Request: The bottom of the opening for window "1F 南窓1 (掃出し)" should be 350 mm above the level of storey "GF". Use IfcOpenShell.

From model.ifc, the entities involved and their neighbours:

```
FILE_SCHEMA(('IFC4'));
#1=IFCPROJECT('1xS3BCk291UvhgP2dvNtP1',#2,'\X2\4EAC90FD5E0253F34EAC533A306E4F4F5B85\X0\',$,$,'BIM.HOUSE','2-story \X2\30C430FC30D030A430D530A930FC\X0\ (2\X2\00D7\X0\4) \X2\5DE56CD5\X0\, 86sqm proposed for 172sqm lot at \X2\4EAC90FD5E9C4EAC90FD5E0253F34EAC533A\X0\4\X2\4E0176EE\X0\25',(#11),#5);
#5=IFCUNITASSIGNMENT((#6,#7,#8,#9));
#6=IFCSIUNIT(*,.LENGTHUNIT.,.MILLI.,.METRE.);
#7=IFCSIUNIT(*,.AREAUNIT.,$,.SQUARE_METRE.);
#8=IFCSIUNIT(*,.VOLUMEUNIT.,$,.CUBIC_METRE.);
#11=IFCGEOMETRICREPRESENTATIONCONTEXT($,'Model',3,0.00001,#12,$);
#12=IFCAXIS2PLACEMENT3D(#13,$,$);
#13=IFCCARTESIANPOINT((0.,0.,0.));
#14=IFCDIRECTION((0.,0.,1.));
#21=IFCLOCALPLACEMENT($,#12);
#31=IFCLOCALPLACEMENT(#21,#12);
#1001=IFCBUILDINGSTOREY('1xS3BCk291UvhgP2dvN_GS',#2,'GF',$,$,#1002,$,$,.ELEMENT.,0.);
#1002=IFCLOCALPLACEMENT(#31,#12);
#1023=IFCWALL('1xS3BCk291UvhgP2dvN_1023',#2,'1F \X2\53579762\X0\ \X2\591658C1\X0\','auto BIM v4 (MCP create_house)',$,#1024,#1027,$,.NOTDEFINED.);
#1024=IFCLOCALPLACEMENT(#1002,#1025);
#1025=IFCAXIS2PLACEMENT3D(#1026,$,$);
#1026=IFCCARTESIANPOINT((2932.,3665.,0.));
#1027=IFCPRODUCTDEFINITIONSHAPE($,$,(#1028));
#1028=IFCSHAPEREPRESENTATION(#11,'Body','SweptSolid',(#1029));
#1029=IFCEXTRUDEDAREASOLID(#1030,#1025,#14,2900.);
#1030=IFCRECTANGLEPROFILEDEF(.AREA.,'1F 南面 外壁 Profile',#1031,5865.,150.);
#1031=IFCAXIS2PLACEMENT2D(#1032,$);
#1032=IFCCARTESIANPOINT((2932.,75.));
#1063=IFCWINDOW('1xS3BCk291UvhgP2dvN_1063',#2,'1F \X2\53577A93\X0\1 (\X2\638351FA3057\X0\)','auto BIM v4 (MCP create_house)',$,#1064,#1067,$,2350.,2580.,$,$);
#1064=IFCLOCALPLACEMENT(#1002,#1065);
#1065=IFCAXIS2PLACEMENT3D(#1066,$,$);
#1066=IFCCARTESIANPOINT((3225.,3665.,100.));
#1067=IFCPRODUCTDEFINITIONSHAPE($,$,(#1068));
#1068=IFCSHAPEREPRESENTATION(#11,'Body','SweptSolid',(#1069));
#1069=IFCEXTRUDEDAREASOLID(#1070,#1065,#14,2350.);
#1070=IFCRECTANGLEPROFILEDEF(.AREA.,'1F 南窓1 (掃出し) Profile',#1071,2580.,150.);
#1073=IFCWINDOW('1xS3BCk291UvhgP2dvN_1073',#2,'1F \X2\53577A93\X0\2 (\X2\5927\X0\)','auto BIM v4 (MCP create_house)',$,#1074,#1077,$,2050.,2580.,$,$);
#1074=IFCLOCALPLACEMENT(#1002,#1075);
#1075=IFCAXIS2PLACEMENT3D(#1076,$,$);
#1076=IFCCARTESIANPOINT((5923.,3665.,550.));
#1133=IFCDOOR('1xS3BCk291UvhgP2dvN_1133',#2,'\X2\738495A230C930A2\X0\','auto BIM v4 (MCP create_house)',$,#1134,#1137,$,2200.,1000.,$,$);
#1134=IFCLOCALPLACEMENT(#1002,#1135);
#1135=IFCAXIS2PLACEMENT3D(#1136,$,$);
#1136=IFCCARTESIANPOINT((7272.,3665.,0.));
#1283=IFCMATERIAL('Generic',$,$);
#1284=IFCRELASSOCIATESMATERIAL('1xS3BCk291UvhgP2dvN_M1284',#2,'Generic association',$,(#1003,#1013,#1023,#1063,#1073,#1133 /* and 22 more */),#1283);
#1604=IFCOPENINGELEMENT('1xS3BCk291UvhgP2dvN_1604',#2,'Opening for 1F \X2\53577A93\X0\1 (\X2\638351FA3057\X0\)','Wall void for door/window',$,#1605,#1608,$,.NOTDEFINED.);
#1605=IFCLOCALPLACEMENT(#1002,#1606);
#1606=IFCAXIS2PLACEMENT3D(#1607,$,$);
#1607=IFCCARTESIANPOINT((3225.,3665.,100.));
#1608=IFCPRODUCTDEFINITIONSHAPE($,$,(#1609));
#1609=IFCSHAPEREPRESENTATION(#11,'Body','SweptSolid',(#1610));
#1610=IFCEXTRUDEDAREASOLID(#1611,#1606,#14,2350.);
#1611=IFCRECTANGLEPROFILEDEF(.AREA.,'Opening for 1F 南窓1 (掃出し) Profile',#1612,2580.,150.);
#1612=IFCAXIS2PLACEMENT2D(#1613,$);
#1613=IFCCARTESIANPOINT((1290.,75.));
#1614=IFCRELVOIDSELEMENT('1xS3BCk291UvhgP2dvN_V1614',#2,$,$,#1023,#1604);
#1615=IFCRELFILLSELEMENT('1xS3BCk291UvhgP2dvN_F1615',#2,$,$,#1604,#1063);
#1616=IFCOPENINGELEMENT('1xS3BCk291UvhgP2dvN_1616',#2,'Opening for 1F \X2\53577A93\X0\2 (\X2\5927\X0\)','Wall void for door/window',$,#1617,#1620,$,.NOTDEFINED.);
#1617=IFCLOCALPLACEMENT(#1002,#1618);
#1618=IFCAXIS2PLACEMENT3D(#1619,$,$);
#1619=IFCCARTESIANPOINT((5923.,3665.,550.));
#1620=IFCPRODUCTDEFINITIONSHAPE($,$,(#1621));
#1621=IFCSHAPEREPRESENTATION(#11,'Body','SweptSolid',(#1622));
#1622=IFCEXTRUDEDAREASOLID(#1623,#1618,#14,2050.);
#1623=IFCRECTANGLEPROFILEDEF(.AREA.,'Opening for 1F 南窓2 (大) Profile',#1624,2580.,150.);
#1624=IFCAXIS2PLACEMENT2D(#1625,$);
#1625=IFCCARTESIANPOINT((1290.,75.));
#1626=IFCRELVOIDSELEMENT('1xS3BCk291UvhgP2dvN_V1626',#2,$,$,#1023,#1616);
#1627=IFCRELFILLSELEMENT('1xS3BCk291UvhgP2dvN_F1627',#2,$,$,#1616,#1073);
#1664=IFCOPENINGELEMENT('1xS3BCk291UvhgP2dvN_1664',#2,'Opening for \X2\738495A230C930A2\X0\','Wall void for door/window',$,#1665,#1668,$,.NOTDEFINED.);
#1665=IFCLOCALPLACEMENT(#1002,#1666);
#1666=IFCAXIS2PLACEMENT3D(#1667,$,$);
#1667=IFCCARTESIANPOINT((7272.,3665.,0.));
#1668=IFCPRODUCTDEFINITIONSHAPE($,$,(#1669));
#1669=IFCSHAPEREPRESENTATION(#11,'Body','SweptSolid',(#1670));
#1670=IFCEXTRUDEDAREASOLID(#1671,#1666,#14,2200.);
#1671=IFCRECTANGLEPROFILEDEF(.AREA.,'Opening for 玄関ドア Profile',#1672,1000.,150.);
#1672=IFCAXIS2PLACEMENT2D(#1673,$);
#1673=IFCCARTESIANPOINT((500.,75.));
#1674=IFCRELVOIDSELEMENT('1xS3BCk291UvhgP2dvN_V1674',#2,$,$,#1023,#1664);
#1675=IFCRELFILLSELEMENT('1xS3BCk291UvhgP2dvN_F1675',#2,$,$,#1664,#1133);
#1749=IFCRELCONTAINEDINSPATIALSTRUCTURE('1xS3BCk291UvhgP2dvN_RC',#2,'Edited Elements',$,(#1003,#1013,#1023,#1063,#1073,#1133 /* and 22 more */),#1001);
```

```python
import numpy as np
import ifcopenshell
import ifcopenshell.api.geometry
import ifcopenshell.geom
import ifcopenshell.util.element
import ifcopenshell.util.placement
import ifcopenshell.util.shape
import ifcopenshell.util.unit

model = ifcopenshell.open("model.ifc")
unit_scale = ifcopenshell.util.unit.calculate_unit_scale(model)

window = model.by_guid("1xS3BCk291UvhgP2dvN_1063")
opening = window.FillsVoids[0].RelatingOpeningElement
storey = ifcopenshell.util.element.get_container(window, ifc_class="IfcBuildingStorey")
level = ifcopenshell.util.placement.get_local_placement(storey.ObjectPlacement)[2, 3]

# The opening's origin need not be at the sill, so measure its lowest point.
shape = ifcopenshell.geom.create_shape(ifcopenshell.geom.settings(), opening)
bottom = ifcopenshell.util.shape.get_shape_bottom_elevation(shape, shape.geometry) / unit_scale
dz = level + 350.0 - bottom

shift = np.array([0.0, 0.0, dz])
# The window is not placed relative to its opening, so move both.
for product in (opening, window):
    matrix = ifcopenshell.util.placement.get_local_placement(product.ObjectPlacement)
    matrix[:3, 3] += shift
    ifcopenshell.api.geometry.edit_object_placement(model, product=product, matrix=matrix, is_si=False)

print(f"moved by {dz * unit_scale:+.3f} m")

model.write("model-out.ifc")
```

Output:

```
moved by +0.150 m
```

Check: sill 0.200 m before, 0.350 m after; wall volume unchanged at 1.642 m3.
